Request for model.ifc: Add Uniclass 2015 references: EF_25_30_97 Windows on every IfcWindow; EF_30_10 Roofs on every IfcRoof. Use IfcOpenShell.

First a look at what the model holds.

```python
import ifcopenshell

model = ifcopenshell.open("model.ifc")
print(model.schema)
print("classifications:", [c.Name for c in model.by_type("IfcClassification")])
for ifc_class in ("IfcDoor", "IfcRoof", "IfcStair", "IfcWall", "IfcWindow"):
    print(ifc_class, len(model.by_type(ifc_class)))
```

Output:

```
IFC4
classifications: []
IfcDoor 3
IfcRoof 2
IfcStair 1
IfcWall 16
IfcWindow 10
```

```python
import ifcopenshell
import ifcopenshell.api.classification

model = ifcopenshell.open("model.ifc")

system = ifcopenshell.api.classification.add_classification(model, classification="Uniclass 2015")

codes = {
    "IfcWindow": ("EF_25_30_97", "Windows"),
    "IfcRoof": ("EF_30_10", "Roofs"),
}
for ifc_class, (code, name) in codes.items():
    products = model.by_type(ifc_class)
    ifcopenshell.api.classification.add_reference(
        model, products=products, classification=system, identification=code, name=name
    )
    print(code, len(products))

model.write("model_edited.ifc")
```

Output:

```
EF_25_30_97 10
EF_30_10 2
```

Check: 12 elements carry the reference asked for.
